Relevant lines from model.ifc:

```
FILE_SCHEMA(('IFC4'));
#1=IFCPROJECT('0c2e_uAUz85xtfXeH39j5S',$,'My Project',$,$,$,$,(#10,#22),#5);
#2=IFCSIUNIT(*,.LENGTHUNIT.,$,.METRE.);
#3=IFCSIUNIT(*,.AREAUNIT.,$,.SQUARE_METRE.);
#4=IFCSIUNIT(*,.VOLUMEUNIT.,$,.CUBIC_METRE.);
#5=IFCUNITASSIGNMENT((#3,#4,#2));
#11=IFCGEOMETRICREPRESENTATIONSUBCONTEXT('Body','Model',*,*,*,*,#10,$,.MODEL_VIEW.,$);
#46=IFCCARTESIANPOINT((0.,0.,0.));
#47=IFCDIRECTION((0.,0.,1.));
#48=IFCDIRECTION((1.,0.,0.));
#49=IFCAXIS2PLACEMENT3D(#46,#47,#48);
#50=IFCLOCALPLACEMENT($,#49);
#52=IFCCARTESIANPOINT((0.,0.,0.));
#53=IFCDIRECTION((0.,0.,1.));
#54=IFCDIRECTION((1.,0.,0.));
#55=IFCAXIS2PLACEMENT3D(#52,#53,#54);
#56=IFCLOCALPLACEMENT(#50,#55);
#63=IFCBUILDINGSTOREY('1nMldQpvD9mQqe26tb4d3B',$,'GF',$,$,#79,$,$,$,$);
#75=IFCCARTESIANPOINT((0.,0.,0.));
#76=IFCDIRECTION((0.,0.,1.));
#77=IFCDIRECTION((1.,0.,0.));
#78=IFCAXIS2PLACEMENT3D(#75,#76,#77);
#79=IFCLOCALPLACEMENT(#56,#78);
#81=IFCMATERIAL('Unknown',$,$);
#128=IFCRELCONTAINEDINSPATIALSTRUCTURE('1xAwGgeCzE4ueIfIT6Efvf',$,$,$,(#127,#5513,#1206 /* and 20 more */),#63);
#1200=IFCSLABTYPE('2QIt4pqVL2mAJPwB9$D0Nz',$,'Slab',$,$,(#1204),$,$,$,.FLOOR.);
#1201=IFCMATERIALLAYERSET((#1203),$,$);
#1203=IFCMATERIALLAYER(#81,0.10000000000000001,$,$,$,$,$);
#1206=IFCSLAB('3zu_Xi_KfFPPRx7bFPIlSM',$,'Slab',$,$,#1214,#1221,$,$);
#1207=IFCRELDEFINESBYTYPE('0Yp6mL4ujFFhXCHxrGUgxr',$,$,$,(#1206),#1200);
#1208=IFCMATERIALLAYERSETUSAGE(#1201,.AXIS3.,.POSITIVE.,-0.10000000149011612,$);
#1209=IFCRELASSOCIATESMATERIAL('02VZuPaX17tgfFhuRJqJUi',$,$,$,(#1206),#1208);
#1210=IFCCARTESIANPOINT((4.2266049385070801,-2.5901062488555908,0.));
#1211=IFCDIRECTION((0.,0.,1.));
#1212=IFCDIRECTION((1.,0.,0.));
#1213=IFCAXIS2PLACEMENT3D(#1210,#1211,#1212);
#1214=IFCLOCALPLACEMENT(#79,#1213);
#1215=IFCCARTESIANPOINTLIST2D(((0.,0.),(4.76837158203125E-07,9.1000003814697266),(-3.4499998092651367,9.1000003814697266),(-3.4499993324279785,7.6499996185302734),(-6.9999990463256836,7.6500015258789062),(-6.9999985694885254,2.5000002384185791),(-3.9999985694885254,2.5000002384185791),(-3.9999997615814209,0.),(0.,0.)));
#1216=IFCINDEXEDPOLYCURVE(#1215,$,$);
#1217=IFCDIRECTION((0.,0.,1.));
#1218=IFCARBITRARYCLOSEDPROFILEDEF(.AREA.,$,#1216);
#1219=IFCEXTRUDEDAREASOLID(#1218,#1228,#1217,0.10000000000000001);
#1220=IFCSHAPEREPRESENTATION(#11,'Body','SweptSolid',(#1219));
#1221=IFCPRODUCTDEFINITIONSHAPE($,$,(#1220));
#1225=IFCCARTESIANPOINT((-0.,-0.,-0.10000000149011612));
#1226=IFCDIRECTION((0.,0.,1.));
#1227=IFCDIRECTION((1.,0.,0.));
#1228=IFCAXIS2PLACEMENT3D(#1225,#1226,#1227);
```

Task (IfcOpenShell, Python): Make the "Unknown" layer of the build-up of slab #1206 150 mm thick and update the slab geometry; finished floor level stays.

```python
import ifcopenshell
import ifcopenshell.util.element
import ifcopenshell.util.representation
import ifcopenshell.util.unit

model = ifcopenshell.open("model.ifc")
unit_scale = ifcopenshell.util.unit.calculate_unit_scale(model)

layer_set = model.by_id(1201)
layer = next(l for l in layer_set.MaterialLayers if l.Material and l.Material.Name == "Unknown")
change = 0.15 / unit_scale - layer.LayerThickness
layer.LayerThickness += change

# Geometry does not follow the layer set by itself.
slabs = [e for e in ifcopenshell.util.element.get_elements_by_material(model, layer_set) if e.is_a("IfcSlab")]
for slab in sorted(slabs, key=lambda e: e.id()):
    body = ifcopenshell.util.representation.get_representation(slab, "Model", "Body")
    solid = body.Items[0]
    old_depth = solid.Depth
    solid.Depth += change
    # Extruded upwards: lower the start of the extrusion so the top stays.
    x, y, z = solid.Position.Location.Coordinates
    solid.Position.Location = model.createIfcCartesianPoint((x, y, z - change))
    print(slab.id(), f"{old_depth:g} -> {solid.Depth:g}")

# The layers are counted up from the underside, which has moved.
for usage in {ifcopenshell.util.element.get_material(slab) for slab in slabs}:
    usage.OffsetFromReferenceLine -= change

model.write("model-out.ifc")
```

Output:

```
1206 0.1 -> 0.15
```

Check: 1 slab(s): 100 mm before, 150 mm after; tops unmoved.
